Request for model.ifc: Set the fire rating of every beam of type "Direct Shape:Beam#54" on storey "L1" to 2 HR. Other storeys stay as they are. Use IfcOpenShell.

First a look at what the model holds.

```python
import ifcopenshell
import ifcopenshell.util.element

model = ifcopenshell.open("model.ifc")
print(model.schema)
storey = next(s for s in model.by_type("IfcBuildingStorey") if s.Name == "L1")
beams = [e for e in ifcopenshell.util.element.get_decomposition(storey) if e.is_a("IfcBeam")]
seen = {}
for e in beams:
    element_type = ifcopenshell.util.element.get_type(e)
    key = (element_type.Name if element_type != e and element_type else None, ifcopenshell.util.element.get_pset(e, "Pset_BeamCommon", "FireRating"))
    seen[key] = seen.get(key, 0) + 1
for (name, value), count in sorted(seen.items(), key=str):
    print(count, "x", name, "|", value)
```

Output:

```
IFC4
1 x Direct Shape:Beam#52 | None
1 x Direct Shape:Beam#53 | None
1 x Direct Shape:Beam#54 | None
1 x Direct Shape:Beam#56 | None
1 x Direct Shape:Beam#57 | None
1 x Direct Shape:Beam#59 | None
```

```python
import ifcopenshell
import ifcopenshell.api.pset
import ifcopenshell.util.element

model = ifcopenshell.open("model.ifc")

storey = next(s for s in model.by_type("IfcBuildingStorey") if s.Name == "L1")
beams = [e for e in ifcopenshell.util.element.get_decomposition(storey) if e.is_a("IfcBeam")]

count = 0
for e in beams:
    element_type = ifcopenshell.util.element.get_type(e)
    if element_type in (None, e) or element_type.Name != "Direct Shape:Beam#54":
        continue
    # add_pset returns the element's existing set when there is one.
    pset = ifcopenshell.api.pset.add_pset(model, product=e, name="Pset_BeamCommon")
    ifcopenshell.api.pset.edit_pset(model, pset=pset, properties={"FireRating": "2 HR"})
    count += 1

print(count, "beams updated")

model.write("model_edited.ifc")
```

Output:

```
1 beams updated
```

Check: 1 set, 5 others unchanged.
